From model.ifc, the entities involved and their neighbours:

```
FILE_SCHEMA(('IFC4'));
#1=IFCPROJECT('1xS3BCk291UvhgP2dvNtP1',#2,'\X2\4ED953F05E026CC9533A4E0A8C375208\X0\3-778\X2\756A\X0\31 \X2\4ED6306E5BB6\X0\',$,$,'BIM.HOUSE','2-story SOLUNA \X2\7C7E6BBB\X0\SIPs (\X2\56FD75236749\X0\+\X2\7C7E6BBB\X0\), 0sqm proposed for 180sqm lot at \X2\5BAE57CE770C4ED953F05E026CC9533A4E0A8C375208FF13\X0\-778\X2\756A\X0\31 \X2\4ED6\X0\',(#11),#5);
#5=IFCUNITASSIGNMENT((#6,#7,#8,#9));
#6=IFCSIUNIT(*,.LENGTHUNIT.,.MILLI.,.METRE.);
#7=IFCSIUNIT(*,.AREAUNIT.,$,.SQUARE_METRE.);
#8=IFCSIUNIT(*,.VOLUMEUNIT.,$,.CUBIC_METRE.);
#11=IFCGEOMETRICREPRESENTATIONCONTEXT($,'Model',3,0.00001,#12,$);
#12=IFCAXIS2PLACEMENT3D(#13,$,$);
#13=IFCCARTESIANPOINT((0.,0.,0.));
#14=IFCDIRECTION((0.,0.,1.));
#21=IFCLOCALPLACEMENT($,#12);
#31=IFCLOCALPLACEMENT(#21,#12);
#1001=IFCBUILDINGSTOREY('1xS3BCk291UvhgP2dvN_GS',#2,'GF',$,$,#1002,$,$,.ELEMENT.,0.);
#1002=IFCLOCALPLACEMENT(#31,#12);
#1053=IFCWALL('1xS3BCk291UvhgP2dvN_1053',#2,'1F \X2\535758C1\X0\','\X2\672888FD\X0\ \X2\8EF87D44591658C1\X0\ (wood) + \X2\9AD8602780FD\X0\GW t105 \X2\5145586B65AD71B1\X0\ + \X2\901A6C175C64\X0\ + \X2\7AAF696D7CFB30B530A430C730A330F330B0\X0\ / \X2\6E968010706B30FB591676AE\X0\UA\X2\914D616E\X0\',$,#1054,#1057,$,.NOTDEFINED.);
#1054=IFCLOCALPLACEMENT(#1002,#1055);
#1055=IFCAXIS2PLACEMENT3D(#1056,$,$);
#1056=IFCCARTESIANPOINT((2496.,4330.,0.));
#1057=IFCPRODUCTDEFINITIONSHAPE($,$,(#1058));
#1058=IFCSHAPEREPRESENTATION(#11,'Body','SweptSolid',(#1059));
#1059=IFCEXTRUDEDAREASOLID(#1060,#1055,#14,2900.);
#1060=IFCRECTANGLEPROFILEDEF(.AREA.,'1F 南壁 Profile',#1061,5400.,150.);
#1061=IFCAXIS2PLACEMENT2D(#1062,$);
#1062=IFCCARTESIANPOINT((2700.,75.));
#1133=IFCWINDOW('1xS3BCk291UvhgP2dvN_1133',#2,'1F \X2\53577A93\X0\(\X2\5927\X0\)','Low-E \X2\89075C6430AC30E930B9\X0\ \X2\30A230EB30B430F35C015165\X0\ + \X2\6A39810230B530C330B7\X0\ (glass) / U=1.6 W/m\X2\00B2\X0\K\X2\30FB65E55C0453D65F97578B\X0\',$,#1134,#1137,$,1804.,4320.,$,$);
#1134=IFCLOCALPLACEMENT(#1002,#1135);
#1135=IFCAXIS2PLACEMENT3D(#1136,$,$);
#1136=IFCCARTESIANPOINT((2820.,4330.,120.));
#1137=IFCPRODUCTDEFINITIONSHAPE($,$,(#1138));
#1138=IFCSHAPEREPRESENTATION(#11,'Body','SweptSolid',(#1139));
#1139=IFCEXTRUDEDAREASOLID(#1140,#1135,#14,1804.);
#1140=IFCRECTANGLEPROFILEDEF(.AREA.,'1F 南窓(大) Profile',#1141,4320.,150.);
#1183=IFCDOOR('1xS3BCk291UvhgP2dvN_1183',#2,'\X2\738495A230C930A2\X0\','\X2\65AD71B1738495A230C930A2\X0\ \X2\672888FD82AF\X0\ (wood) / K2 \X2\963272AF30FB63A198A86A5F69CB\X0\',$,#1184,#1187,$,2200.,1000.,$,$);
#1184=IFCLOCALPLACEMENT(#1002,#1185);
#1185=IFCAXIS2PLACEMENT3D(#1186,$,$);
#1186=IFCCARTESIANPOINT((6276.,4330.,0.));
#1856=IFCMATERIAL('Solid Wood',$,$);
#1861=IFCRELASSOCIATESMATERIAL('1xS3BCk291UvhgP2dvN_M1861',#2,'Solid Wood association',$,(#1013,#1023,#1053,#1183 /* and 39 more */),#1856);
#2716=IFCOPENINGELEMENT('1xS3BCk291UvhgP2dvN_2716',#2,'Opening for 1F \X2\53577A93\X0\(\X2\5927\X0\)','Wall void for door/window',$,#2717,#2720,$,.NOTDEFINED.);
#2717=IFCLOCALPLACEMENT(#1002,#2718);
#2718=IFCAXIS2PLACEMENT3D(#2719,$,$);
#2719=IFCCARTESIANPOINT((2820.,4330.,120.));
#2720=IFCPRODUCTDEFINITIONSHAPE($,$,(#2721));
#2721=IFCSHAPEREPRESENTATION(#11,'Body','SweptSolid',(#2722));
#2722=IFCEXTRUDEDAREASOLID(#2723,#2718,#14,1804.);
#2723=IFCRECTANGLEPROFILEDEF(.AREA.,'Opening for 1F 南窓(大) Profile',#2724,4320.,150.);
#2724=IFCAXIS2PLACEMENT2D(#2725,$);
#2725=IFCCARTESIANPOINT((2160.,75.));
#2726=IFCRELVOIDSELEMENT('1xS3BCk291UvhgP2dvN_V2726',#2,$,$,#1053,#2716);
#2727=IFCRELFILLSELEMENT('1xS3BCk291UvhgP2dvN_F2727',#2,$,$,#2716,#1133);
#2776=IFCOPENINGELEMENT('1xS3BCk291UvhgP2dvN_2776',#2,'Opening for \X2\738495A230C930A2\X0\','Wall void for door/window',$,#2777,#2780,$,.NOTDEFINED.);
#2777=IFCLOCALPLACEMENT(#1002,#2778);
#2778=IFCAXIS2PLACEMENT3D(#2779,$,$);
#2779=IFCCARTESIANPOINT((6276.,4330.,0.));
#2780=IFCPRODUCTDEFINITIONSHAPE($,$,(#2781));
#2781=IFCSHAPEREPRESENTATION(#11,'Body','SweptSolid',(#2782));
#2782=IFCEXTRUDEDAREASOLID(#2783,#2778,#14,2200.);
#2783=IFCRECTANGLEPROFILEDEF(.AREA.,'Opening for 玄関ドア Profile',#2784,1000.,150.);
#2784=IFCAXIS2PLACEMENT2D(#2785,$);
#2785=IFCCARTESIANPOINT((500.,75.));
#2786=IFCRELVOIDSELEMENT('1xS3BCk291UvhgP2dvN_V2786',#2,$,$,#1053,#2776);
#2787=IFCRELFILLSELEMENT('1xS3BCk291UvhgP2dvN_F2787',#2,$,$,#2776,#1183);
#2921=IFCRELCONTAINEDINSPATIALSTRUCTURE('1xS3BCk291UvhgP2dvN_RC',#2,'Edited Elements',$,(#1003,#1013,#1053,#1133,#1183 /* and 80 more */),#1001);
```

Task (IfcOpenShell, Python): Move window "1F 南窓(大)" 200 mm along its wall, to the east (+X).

```python
import ifcopenshell
import ifcopenshell.api.geometry
import ifcopenshell.util.placement
import ifcopenshell.util.unit

model = ifcopenshell.open("model.ifc")
unit_scale = ifcopenshell.util.unit.calculate_unit_scale(model)

window = model.by_id(1133)
opening = window.FillsVoids[0].RelatingOpeningElement
wall = opening.VoidsElements[0].RelatingBuildingElement

wall_matrix = ifcopenshell.util.placement.get_local_placement(wall.ObjectPlacement)
shift = wall_matrix[:3, 0] * 0.2 / unit_scale
before = ifcopenshell.util.placement.get_local_placement(window.ObjectPlacement)[:3, 3].copy()

# The window is not placed relative to its opening, so move both.
for product in (opening, window):
    matrix = ifcopenshell.util.placement.get_local_placement(product.ObjectPlacement)
    matrix[:3, 3] += shift
    ifcopenshell.api.geometry.edit_object_placement(model, product=product, matrix=matrix, is_si=False)

after = ifcopenshell.util.placement.get_local_placement(window.ObjectPlacement)[:3, 3]
print("window moved by", (after - before).round(3) + 0.0)

model.write("model_rev.ifc")
```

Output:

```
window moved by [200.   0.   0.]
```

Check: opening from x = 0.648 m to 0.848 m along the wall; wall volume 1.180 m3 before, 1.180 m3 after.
